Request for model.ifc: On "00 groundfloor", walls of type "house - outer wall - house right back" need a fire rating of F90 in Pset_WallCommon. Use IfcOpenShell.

First a look at what the model holds.

```python
import ifcopenshell
import ifcopenshell.util.element

model = ifcopenshell.open("model.ifc")
print(model.schema)
storey = next(s for s in model.by_type("IfcBuildingStorey") if s.Name == "00 groundfloor")
walls = [e for e in ifcopenshell.util.element.get_decomposition(storey) if e.is_a("IfcWall")]
seen = {}
for e in walls:
    element_type = ifcopenshell.util.element.get_type(e)
    key = (element_type.Name if element_type != e and element_type else None, ifcopenshell.util.element.get_pset(e, "Pset_WallCommon", "FireRating"))
    seen[key] = seen.get(key, 0) + 1
for (name, value), count in sorted(seen.items(), key=str):
    print(count, "x", name, "|", value)
```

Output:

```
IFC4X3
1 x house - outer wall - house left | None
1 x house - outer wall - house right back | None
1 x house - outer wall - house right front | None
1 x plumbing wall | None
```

```python
import ifcopenshell
import ifcopenshell.api.pset
import ifcopenshell.util.element

model = ifcopenshell.open("model.ifc")

storey = next(s for s in model.by_type("IfcBuildingStorey") if s.Name == "00 groundfloor")
walls = [e for e in ifcopenshell.util.element.get_decomposition(storey) if e.is_a("IfcWall")]

count = 0
for e in walls:
    element_type = ifcopenshell.util.element.get_type(e)
    if element_type in (None, e) or element_type.Name != "house - outer wall - house right back":
        continue
    # add_pset returns the element's existing set when there is one.
    pset = ifcopenshell.api.pset.add_pset(model, product=e, name="Pset_WallCommon")
    ifcopenshell.api.pset.edit_pset(model, pset=pset, properties={"FireRating": "F90"})
    count += 1

print(count, "walls updated")

model.write("model_updated.ifc")
```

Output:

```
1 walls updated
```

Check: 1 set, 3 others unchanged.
